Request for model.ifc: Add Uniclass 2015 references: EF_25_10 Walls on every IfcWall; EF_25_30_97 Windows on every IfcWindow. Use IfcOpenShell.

First a look at what the model holds.

```python
import ifcopenshell

model = ifcopenshell.open("model.ifc")
print(model.schema)
print("classifications:", [c.Name for c in model.by_type("IfcClassification")])
for ifc_class in ("IfcDoor", "IfcRoof", "IfcStair", "IfcWall", "IfcWindow"):
    print(ifc_class, len(model.by_type(ifc_class)))
```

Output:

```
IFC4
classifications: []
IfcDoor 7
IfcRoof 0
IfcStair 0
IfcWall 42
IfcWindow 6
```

```python
import ifcopenshell
import ifcopenshell.api.classification

model = ifcopenshell.open("model.ifc")

system = ifcopenshell.api.classification.add_classification(model, classification="Uniclass 2015")

codes = {
    "IfcWall": ("EF_25_10", "Walls"),
    "IfcWindow": ("EF_25_30_97", "Windows"),
}
for ifc_class, (code, name) in codes.items():
    products = model.by_type(ifc_class)
    ifcopenshell.api.classification.add_reference(
        model, products=products, classification=system, identification=code, name=name
    )
    print(code, len(products))

model.write("model_v2.ifc")
```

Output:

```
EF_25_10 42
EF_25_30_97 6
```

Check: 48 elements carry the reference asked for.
